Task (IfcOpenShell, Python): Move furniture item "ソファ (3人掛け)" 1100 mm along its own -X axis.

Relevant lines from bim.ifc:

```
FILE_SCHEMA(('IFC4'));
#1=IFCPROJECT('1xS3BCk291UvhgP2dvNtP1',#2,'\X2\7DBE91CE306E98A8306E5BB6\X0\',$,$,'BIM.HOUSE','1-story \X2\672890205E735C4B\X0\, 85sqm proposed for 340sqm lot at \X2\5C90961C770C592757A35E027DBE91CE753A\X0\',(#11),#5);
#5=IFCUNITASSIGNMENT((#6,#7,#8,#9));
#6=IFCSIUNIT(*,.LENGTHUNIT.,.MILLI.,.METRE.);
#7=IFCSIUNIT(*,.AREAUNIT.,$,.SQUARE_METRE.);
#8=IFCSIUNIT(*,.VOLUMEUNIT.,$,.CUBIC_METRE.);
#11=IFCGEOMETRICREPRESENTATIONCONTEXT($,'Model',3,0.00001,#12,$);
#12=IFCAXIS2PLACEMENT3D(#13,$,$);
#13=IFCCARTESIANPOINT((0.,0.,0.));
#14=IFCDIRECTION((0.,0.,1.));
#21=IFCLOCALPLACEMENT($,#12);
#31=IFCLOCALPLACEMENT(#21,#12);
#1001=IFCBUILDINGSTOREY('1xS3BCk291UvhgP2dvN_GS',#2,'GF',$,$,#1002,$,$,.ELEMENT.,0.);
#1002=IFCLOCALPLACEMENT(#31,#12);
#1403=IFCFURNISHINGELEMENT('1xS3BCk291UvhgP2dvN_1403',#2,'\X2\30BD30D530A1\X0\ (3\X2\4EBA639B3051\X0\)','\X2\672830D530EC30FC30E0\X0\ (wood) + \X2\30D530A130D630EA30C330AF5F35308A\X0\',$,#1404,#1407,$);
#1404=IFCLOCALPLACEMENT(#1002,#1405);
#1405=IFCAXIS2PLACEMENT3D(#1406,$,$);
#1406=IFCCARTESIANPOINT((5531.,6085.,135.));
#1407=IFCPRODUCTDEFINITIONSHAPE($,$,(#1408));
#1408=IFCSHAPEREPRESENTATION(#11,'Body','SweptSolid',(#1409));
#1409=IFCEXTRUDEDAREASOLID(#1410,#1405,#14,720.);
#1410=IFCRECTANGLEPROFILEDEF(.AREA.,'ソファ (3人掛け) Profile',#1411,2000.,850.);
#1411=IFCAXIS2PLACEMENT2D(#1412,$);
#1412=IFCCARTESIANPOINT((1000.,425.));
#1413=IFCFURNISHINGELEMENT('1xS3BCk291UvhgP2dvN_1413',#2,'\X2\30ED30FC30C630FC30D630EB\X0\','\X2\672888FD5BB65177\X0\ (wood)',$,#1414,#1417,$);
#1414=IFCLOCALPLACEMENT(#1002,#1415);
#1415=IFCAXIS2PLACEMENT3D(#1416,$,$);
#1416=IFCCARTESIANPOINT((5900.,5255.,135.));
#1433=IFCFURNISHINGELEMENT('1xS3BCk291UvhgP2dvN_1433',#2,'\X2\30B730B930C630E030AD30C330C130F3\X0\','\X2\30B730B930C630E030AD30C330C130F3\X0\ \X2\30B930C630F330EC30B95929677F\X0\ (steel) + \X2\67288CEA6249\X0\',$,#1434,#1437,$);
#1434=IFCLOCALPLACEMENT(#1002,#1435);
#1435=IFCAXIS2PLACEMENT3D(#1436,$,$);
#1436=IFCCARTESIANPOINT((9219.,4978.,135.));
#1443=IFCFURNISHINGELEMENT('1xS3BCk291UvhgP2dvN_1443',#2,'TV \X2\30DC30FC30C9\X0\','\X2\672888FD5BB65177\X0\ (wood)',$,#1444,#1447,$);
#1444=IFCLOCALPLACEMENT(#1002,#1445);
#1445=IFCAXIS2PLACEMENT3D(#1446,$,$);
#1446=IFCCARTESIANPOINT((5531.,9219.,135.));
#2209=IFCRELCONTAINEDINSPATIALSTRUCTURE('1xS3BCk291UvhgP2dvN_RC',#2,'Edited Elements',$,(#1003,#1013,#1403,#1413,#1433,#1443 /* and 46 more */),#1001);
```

```python
import ifcopenshell
import ifcopenshell.api.geometry
import ifcopenshell.util.placement

model = ifcopenshell.open("bim.ifc")

item = model.by_guid("1xS3BCk291UvhgP2dvN_1403")
matrix = ifcopenshell.util.placement.get_local_placement(item.ObjectPlacement)
matrix[:3, 3] -= matrix[:3, 0] * 1100.0
ifcopenshell.api.geometry.edit_object_placement(model, product=item, matrix=matrix, is_si=False)

print(ifcopenshell.util.placement.get_local_placement(item.ObjectPlacement).round(3) + 0.0)

model.write("bim_updated.ifc")
```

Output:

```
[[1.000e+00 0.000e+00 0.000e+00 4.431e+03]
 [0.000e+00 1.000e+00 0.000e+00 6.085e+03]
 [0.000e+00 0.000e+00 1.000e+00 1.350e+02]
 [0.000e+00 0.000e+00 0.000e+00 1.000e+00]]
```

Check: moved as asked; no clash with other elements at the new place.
